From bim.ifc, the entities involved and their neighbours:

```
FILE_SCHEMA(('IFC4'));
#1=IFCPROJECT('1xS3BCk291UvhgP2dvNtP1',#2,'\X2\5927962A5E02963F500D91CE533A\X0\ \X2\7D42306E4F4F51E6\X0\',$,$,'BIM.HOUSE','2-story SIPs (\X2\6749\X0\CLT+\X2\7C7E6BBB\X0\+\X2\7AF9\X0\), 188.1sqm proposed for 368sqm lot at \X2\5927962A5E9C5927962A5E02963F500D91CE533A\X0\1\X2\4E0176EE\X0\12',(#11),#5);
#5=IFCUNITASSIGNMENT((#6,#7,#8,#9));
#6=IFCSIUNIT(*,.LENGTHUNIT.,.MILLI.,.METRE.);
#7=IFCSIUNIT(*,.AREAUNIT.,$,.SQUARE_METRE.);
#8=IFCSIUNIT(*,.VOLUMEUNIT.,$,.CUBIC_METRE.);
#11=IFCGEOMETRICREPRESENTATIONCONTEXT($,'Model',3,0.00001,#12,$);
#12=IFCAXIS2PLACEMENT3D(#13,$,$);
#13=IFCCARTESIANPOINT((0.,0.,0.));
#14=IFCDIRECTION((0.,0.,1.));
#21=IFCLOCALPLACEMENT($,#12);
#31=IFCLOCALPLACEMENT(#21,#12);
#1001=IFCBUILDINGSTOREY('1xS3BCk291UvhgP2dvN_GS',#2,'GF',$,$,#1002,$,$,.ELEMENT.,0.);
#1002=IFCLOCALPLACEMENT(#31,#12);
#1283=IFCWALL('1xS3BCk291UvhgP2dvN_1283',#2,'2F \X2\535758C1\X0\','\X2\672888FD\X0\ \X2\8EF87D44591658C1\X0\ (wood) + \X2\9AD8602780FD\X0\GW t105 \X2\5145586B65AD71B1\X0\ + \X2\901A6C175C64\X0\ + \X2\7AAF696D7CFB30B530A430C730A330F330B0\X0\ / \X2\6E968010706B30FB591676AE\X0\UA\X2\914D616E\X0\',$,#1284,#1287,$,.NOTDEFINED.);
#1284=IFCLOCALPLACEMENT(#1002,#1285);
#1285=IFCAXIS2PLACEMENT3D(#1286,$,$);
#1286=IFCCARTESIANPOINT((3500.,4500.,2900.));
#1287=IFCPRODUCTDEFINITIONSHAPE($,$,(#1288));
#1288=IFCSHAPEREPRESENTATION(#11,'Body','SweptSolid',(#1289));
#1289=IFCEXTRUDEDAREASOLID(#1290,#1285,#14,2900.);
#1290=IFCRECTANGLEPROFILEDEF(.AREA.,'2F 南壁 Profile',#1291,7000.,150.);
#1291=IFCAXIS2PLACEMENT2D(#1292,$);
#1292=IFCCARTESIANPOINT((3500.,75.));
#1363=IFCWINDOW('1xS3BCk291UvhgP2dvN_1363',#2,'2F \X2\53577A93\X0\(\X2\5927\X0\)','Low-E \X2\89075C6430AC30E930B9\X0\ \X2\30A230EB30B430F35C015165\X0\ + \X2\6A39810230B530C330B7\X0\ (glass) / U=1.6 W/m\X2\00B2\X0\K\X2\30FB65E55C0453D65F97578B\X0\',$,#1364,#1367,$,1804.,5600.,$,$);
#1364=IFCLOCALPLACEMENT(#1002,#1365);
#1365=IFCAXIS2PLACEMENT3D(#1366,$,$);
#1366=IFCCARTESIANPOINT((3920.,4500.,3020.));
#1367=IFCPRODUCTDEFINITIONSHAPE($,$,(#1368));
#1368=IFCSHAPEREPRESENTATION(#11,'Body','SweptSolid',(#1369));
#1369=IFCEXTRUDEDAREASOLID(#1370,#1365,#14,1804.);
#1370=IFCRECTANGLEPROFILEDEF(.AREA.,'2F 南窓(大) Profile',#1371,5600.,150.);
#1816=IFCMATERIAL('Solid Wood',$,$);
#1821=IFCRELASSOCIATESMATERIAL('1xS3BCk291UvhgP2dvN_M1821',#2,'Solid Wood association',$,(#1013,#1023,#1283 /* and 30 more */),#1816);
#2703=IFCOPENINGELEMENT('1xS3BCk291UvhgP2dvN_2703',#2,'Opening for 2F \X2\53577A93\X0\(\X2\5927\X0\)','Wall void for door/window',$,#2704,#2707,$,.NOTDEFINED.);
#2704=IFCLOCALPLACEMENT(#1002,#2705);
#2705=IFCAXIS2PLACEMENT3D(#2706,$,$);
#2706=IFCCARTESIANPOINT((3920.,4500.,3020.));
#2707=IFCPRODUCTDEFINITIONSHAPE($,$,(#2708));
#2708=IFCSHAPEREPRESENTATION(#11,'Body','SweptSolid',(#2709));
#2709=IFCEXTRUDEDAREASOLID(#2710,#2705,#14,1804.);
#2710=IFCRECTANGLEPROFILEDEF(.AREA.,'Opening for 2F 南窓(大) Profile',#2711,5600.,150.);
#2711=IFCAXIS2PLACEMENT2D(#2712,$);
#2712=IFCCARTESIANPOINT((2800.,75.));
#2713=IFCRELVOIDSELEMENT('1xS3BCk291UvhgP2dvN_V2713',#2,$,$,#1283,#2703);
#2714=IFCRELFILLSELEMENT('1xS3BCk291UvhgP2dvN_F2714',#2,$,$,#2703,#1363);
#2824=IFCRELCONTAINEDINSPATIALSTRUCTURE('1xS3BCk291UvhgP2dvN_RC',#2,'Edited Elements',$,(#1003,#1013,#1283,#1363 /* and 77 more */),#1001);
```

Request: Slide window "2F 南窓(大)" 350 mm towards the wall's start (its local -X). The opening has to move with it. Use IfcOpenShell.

```python
import ifcopenshell
import ifcopenshell.api.geometry
import ifcopenshell.util.placement
import ifcopenshell.util.unit

model = ifcopenshell.open("bim.ifc")
unit_scale = ifcopenshell.util.unit.calculate_unit_scale(model)

window = model.by_guid("1xS3BCk291UvhgP2dvN_1363")
opening = window.FillsVoids[0].RelatingOpeningElement
wall = opening.VoidsElements[0].RelatingBuildingElement

wall_matrix = ifcopenshell.util.placement.get_local_placement(wall.ObjectPlacement)
shift = wall_matrix[:3, 0] * -0.35 / unit_scale
before = ifcopenshell.util.placement.get_local_placement(window.ObjectPlacement)[:3, 3].copy()

# The window is not placed relative to its opening, so move both.
for product in (opening, window):
    matrix = ifcopenshell.util.placement.get_local_placement(product.ObjectPlacement)
    matrix[:3, 3] += shift
    ifcopenshell.api.geometry.edit_object_placement(model, product=product, matrix=matrix, is_si=False)

after = ifcopenshell.util.placement.get_local_placement(window.ObjectPlacement)[:3, 3]
print("window moved by", (after - before).round(3) + 0.0)

model.write("bim_v2.ifc")
```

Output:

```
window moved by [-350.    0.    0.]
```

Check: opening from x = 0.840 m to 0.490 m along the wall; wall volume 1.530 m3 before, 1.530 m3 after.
